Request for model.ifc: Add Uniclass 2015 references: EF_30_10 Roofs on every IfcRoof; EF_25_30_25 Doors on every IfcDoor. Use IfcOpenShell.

First a look at what the model holds.

```python
import ifcopenshell

model = ifcopenshell.open("model.ifc")
print(model.schema)
print("classifications:", [c.Name for c in model.by_type("IfcClassification")])
for ifc_class in ("IfcDoor", "IfcRoof", "IfcStair", "IfcWall", "IfcWindow"):
    print(ifc_class, len(model.by_type(ifc_class)))
```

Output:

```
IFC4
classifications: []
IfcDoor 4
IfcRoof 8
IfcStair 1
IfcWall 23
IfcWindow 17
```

```python
import ifcopenshell
import ifcopenshell.api.classification

model = ifcopenshell.open("model.ifc")

system = ifcopenshell.api.classification.add_classification(model, classification="Uniclass 2015")

codes = {
    "IfcRoof": ("EF_30_10", "Roofs"),
    "IfcDoor": ("EF_25_30_25", "Doors"),
}
for ifc_class, (code, name) in codes.items():
    products = model.by_type(ifc_class)
    ifcopenshell.api.classification.add_reference(
        model, products=products, classification=system, identification=code, name=name
    )
    print(code, len(products))

model.write("model_updated.ifc")
```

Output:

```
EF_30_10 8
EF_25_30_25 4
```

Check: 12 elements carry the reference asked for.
